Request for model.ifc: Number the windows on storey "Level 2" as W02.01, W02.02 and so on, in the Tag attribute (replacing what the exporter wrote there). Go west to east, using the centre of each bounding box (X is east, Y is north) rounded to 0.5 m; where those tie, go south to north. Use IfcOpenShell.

First a look at what the model holds.

```python
import ifcopenshell
import ifcopenshell.util.element
import ifcopenshell.util.placement

model = ifcopenshell.open("model.ifc")
print(model.schema)
storey = next(s for s in model.by_type("IfcBuildingStorey") if s.Name == "Level 2")
windows = [e for e in ifcopenshell.util.element.get_decomposition(storey) if e.is_a("IfcWindow")]
for e in sorted(windows, key=lambda e: e.id()):
    origin = ifcopenshell.util.placement.get_local_placement(e.ObjectPlacement)[:3, 3]
    print(e.id(), e.Tag, e.Name, origin.round(2) + 0.0, sep=" | ")
```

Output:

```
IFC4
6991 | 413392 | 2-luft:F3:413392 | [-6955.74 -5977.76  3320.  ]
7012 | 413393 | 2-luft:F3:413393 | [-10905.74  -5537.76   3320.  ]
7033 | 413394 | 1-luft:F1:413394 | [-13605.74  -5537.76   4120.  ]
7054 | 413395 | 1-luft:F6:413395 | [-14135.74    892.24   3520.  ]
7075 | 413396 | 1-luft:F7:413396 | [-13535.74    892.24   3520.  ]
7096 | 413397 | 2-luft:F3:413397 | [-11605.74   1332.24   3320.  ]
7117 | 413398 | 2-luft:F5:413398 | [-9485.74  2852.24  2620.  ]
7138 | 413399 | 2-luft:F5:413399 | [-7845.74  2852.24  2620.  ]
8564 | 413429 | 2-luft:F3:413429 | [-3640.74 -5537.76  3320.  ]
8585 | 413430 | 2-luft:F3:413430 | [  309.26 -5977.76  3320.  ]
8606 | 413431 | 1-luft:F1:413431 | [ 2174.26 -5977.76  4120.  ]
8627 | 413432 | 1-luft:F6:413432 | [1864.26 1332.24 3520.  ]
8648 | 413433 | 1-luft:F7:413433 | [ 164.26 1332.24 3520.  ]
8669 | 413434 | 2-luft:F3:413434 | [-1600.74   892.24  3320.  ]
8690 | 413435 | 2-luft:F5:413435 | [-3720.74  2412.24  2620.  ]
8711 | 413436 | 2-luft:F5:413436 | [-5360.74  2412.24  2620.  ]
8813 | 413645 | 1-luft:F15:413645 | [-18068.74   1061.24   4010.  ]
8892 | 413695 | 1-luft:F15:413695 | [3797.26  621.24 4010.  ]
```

```python
import ifcopenshell
import ifcopenshell.geom
import ifcopenshell.util.element
import ifcopenshell.util.shape

model = ifcopenshell.open("model.ifc")
settings = ifcopenshell.geom.settings()
settings.set("use-world-coords", True)


def centre(element):
    shape = ifcopenshell.geom.create_shape(settings, element)
    return ifcopenshell.util.shape.get_bbox_centroid(shape.geometry)


storey = next(s for s in model.by_type("IfcBuildingStorey") if s.Name == "Level 2")
windows = [e for e in ifcopenshell.util.element.get_decomposition(storey) if e.is_a("IfcWindow")]

# Insertion points can sit at a corner or the storey origin, so sort by the geometry (in metres).
centres = {e: centre(e) for e in windows}
windows.sort(key=lambda e: (round(centres[e][0] / 0.5), centres[e][1]))

for i, e in enumerate(windows, start=1):
    number = f"W02.{i:02d}"
    e.Tag = number
    print(e.id(), number)

model.write("model_v2.ifc")
```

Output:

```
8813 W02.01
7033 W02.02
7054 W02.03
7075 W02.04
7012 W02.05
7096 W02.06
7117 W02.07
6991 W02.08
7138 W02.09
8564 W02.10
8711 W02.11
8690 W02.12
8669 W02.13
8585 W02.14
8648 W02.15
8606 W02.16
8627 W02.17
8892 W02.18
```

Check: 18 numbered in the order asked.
